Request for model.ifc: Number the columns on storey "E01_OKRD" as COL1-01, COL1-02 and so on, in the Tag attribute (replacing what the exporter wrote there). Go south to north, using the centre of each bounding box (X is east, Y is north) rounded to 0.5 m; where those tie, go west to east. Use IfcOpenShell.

First a look at what the model holds.

```python
import ifcopenshell
import ifcopenshell.util.element
import ifcopenshell.util.placement

model = ifcopenshell.open("model.ifc")
print(model.schema)
storey = next(s for s in model.by_type("IfcBuildingStorey") if s.Name == "E01_OKRD")
columns = [e for e in ifcopenshell.util.element.get_decomposition(storey) if e.is_a("IfcColumn")]
for e in sorted(columns, key=lambda e: e.id()):
    origin = ifcopenshell.util.placement.get_local_placement(e.ObjectPlacement)[:3, 3]
    print(e.id(), e.Tag, e.Name, origin.round(2) + 0.0, sep=" | ")
```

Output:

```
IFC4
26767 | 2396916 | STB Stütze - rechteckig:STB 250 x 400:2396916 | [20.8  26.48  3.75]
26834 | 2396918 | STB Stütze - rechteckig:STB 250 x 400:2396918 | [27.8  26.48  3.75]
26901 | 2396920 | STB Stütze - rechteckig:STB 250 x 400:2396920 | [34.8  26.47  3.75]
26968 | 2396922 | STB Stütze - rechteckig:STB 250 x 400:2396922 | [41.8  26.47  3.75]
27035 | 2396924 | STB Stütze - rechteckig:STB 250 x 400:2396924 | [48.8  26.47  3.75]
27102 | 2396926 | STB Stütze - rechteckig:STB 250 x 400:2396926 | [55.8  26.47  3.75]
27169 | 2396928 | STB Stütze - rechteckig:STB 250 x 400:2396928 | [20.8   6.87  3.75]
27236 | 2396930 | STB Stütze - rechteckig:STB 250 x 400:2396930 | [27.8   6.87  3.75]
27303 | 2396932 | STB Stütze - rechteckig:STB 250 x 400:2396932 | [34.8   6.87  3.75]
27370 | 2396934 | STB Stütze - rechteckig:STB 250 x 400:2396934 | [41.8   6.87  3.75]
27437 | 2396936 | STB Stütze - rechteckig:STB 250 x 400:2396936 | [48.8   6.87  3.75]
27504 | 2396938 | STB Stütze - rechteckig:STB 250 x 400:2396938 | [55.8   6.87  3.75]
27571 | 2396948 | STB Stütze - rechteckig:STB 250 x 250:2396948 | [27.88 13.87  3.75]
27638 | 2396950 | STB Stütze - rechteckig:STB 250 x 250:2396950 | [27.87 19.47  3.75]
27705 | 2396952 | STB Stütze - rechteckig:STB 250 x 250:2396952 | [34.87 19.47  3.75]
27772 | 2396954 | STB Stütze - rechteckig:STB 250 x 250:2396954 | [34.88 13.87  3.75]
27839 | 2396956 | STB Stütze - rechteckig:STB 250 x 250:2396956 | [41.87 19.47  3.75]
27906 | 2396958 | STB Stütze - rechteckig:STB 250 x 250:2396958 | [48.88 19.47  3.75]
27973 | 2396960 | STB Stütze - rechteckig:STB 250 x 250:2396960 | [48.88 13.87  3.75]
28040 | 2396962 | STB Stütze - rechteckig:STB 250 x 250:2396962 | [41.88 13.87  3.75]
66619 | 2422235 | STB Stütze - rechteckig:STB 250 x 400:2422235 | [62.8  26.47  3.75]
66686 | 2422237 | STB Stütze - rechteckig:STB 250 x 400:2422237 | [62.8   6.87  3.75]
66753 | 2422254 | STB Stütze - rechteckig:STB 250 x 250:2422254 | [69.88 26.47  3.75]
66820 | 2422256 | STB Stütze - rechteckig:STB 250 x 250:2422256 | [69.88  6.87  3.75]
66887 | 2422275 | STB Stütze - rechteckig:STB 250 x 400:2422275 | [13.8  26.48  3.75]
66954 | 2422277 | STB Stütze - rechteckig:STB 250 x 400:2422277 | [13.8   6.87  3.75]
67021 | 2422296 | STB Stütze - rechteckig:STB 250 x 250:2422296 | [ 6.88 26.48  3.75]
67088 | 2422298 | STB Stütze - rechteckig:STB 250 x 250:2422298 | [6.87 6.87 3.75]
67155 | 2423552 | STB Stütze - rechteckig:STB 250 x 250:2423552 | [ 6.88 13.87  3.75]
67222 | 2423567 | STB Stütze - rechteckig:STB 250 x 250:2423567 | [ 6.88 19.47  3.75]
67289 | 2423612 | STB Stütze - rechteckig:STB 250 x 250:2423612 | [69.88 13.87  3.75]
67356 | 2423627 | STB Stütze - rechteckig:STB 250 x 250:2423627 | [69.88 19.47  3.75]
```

```python
import ifcopenshell
import ifcopenshell.geom
import ifcopenshell.util.element
import ifcopenshell.util.shape

model = ifcopenshell.open("model.ifc")
settings = ifcopenshell.geom.settings()
settings.set("use-world-coords", True)


def centre(element):
    shape = ifcopenshell.geom.create_shape(settings, element)
    return ifcopenshell.util.shape.get_bbox_centroid(shape.geometry)


storey = next(s for s in model.by_type("IfcBuildingStorey") if s.Name == "E01_OKRD")
columns = [e for e in ifcopenshell.util.element.get_decomposition(storey) if e.is_a("IfcColumn")]

# Insertion points can sit at a corner or the storey origin, so sort by the geometry (in metres).
centres = {e: centre(e) for e in columns}
columns.sort(key=lambda e: (round(centres[e][1] / 0.5), centres[e][0]))

for i, e in enumerate(columns, start=1):
    number = f"COL1-{i:02d}"
    e.Tag = number
    print(e.id(), number)

model.write("model_rev.ifc")
```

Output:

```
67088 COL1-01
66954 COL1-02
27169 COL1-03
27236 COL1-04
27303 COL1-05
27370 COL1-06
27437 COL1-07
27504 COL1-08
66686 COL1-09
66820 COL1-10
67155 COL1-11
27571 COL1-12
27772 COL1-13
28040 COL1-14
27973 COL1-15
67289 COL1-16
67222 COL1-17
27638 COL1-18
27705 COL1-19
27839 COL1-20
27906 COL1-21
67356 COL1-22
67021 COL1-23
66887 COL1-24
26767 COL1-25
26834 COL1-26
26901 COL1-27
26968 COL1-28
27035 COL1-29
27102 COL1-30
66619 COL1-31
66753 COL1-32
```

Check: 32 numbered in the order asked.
